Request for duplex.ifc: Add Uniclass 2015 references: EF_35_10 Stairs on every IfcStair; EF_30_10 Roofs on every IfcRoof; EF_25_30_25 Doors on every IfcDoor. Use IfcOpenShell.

First a look at what the model holds.

```python
import ifcopenshell

model = ifcopenshell.open("duplex.ifc")
print(model.schema)
print("classifications:", [c.Name for c in model.by_type("IfcClassification")])
for ifc_class in ("IfcDoor", "IfcRoof", "IfcStair", "IfcWall", "IfcWindow"):
    print(ifc_class, len(model.by_type(ifc_class)))
```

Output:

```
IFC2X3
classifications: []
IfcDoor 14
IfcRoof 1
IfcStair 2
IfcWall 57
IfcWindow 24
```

```python
import ifcopenshell
import ifcopenshell.api.classification

model = ifcopenshell.open("duplex.ifc")

# IFC2X3 requires Source and Edition and has no link from the project to the system.
system = model.create_entity("IfcClassification", Source="NBS", Edition="2015", Name="Uniclass 2015")

codes = {
    "IfcStair": ("EF_35_10", "Stairs"),
    "IfcRoof": ("EF_30_10", "Roofs"),
    "IfcDoor": ("EF_25_30_25", "Doors"),
}
for ifc_class, (code, name) in codes.items():
    products = model.by_type(ifc_class)
    ifcopenshell.api.classification.add_reference(
        model, products=products, classification=system, identification=code, name=name
    )
    print(code, len(products))

model.write("duplex_edited.ifc")
```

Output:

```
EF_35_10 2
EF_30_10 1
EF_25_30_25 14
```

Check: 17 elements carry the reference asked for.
